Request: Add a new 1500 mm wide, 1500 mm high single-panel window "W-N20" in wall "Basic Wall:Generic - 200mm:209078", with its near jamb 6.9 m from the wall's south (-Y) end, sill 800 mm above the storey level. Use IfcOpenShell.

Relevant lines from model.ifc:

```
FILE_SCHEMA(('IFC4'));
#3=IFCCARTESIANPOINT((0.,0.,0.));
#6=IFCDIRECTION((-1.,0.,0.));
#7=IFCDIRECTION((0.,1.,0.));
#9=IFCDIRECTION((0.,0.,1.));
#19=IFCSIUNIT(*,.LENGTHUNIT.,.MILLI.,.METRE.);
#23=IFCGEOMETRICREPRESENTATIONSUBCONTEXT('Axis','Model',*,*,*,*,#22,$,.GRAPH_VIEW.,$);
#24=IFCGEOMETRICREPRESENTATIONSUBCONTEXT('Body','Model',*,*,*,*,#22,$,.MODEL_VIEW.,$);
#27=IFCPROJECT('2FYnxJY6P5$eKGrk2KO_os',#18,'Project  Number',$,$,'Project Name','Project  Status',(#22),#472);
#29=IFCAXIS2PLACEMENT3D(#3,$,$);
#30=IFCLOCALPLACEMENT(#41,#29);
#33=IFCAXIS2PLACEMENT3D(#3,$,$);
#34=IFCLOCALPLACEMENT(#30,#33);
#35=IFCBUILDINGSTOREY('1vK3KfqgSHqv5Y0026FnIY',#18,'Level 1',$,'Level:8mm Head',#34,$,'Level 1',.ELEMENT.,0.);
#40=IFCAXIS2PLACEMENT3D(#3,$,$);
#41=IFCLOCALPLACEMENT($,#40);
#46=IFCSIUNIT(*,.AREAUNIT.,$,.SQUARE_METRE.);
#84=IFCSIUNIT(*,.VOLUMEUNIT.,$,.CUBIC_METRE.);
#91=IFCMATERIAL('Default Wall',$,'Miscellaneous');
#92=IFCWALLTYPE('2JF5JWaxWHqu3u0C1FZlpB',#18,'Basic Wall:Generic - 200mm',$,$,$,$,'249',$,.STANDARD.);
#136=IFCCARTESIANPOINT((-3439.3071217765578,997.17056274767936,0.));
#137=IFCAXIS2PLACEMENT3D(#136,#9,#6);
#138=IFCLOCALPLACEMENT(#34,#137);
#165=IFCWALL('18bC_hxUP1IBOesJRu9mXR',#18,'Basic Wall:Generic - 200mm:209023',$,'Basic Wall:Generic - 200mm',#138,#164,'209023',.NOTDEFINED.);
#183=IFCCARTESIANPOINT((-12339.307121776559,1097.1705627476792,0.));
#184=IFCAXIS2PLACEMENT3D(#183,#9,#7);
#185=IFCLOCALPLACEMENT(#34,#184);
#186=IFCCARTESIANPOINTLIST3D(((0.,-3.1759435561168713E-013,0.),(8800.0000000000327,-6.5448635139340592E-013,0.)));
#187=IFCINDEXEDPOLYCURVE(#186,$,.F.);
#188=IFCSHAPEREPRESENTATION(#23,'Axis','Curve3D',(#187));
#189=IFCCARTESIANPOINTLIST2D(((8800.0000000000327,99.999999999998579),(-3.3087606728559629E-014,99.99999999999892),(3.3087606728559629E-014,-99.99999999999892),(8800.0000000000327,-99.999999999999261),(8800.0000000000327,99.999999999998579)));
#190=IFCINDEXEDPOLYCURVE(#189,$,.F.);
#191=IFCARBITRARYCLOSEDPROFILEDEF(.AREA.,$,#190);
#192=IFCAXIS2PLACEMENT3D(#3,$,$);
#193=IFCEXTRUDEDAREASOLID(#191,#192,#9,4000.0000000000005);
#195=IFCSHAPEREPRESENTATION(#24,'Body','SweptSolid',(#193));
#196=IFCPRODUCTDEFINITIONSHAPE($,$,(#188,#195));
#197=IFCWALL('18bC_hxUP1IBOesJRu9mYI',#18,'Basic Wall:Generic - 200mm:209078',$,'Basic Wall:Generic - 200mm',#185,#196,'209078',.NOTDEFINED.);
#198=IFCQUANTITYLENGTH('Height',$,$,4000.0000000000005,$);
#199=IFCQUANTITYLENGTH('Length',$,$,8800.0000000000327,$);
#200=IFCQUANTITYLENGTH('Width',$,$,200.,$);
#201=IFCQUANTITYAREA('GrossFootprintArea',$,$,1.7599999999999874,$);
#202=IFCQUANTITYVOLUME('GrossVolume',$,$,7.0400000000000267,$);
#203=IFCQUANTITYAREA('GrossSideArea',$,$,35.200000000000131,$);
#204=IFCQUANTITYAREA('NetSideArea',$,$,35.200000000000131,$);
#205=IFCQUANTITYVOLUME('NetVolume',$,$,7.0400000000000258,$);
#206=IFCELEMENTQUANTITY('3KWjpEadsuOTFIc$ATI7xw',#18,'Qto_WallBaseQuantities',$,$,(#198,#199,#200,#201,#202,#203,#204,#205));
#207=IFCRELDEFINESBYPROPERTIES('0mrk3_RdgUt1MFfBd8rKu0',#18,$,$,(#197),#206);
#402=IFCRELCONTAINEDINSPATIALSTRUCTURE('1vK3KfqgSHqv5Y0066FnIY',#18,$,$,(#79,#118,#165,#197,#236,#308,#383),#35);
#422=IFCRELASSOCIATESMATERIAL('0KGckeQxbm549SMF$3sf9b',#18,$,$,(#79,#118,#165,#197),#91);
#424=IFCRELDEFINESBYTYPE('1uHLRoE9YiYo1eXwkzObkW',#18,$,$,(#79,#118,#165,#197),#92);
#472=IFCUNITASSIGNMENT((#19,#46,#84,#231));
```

```python
import numpy as np
import ifcopenshell
import ifcopenshell.api.feature
import ifcopenshell.api.geometry
import ifcopenshell.api.pset
import ifcopenshell.api.root
import ifcopenshell.api.spatial
import ifcopenshell.geom
import ifcopenshell.util.element
import ifcopenshell.util.placement
import ifcopenshell.util.representation
import ifcopenshell.util.shape
import ifcopenshell.util.unit

model = ifcopenshell.open("model.ifc")
unit_scale = ifcopenshell.util.unit.calculate_unit_scale(model)
area_scale = ifcopenshell.util.unit.calculate_unit_scale(model, "AREAUNIT")
volume_scale = ifcopenshell.util.unit.calculate_unit_scale(model, "VOLUMEUNIT")
settings = ifcopenshell.geom.settings()


def volume(element):
    """Net volume in cubic metres, openings subtracted."""
    shape = ifcopenshell.geom.create_shape(settings, element)
    return ifcopenshell.util.shape.get_volume(shape.geometry)


wall = model.by_id(197)
storey = ifcopenshell.util.element.get_container(wall, ifc_class="IfcBuildingStorey")
context = ifcopenshell.util.representation.get_context(model, "Model", "Body", "MODEL_VIEW")
before = volume(wall)

width, height, from_end, sill = 1.5, 1.5, 6.9, 0.8  # metres

# The wall runs along its own X axis, and the end named is its -X end.
wall_shape = ifcopenshell.geom.create_shape(settings, wall)
x, y, z = ifcopenshell.util.shape.get_vertices(wall_shape.geometry).T
start = x.min() + from_end
face, thickness = float(y.min()), float(y.max() - y.min())
wall_matrix = ifcopenshell.util.placement.get_local_placement(wall.ObjectPlacement)
level = ifcopenshell.util.placement.get_local_placement(storey.ObjectPlacement)[2, 3]


def in_wall(x, y):
    """Placement at x, y metres in the wall's axes, at sill height."""
    matrix = wall_matrix.copy()
    matrix[:, 3] = wall_matrix @ np.array([x / unit_scale, y / unit_scale, 0.0, 1.0])
    matrix[2, 3] = level + sill / unit_scale
    return matrix


# Opening: a box that overshoots both wall faces by 50 mm.
opening = ifcopenshell.api.root.create_entity(model, ifc_class="IfcOpeningElement", predefined_type="OPENING")
box = ifcopenshell.api.geometry.add_wall_representation(
    model, context=context, length=width, height=height, thickness=thickness + 0.1
)
ifcopenshell.api.geometry.assign_representation(model, product=opening, representation=box)
ifcopenshell.api.geometry.edit_object_placement(model, product=opening, matrix=in_wall(start, face - 0.05), is_si=False)
ifcopenshell.api.feature.add_feature(model, feature=opening, element=wall)

window = ifcopenshell.api.root.create_entity(model, ifc_class="IfcWindow", name="W-N20", predefined_type="WINDOW")
window.OverallWidth, window.OverallHeight = width / unit_scale, height / unit_scale
window.PartitioningType = "SINGLE_PANEL"
body = ifcopenshell.api.geometry.add_window_representation(
    model,
    context=context,
    overall_width=window.OverallWidth,
    overall_height=window.OverallHeight,
    partition_type="SINGLE_PANEL",
)
ifcopenshell.api.geometry.assign_representation(model, product=window, representation=body)
ifcopenshell.api.spatial.assign_container(model, products=[window], relating_structure=storey)
ifcopenshell.api.feature.add_filling(model, opening=opening, element=window)

# Centre the window in the wall's thickness.
ifcopenshell.api.geometry.edit_object_placement(model, product=window, matrix=in_wall(start, face), is_si=False)
window_shape = ifcopenshell.geom.create_shape(settings, window)
depth = ifcopenshell.util.shape.get_vertices(window_shape.geometry)[:, 1]
offset = face + thickness / 2 - (depth.min() + depth.max()) / 2
ifcopenshell.api.geometry.edit_object_placement(model, product=window, matrix=in_wall(start, offset), is_si=False)

after = volume(wall)

# Update the wall's stored quantities.
qto = model.by_id(ifcopenshell.util.element.get_pset(wall, "Qto_WallBaseQuantities", should_inherit=False)["id"])
ifcopenshell.api.pset.edit_qto(model, qto=qto, properties={
    "NetSideArea": after / thickness / area_scale,
    "NetVolume": after / volume_scale,
})

print(f"wall volume {before:.3f} -> {after:.3f} m3")

model.write("model-out.ifc")
```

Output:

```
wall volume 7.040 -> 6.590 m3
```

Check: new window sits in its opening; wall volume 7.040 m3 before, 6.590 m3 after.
